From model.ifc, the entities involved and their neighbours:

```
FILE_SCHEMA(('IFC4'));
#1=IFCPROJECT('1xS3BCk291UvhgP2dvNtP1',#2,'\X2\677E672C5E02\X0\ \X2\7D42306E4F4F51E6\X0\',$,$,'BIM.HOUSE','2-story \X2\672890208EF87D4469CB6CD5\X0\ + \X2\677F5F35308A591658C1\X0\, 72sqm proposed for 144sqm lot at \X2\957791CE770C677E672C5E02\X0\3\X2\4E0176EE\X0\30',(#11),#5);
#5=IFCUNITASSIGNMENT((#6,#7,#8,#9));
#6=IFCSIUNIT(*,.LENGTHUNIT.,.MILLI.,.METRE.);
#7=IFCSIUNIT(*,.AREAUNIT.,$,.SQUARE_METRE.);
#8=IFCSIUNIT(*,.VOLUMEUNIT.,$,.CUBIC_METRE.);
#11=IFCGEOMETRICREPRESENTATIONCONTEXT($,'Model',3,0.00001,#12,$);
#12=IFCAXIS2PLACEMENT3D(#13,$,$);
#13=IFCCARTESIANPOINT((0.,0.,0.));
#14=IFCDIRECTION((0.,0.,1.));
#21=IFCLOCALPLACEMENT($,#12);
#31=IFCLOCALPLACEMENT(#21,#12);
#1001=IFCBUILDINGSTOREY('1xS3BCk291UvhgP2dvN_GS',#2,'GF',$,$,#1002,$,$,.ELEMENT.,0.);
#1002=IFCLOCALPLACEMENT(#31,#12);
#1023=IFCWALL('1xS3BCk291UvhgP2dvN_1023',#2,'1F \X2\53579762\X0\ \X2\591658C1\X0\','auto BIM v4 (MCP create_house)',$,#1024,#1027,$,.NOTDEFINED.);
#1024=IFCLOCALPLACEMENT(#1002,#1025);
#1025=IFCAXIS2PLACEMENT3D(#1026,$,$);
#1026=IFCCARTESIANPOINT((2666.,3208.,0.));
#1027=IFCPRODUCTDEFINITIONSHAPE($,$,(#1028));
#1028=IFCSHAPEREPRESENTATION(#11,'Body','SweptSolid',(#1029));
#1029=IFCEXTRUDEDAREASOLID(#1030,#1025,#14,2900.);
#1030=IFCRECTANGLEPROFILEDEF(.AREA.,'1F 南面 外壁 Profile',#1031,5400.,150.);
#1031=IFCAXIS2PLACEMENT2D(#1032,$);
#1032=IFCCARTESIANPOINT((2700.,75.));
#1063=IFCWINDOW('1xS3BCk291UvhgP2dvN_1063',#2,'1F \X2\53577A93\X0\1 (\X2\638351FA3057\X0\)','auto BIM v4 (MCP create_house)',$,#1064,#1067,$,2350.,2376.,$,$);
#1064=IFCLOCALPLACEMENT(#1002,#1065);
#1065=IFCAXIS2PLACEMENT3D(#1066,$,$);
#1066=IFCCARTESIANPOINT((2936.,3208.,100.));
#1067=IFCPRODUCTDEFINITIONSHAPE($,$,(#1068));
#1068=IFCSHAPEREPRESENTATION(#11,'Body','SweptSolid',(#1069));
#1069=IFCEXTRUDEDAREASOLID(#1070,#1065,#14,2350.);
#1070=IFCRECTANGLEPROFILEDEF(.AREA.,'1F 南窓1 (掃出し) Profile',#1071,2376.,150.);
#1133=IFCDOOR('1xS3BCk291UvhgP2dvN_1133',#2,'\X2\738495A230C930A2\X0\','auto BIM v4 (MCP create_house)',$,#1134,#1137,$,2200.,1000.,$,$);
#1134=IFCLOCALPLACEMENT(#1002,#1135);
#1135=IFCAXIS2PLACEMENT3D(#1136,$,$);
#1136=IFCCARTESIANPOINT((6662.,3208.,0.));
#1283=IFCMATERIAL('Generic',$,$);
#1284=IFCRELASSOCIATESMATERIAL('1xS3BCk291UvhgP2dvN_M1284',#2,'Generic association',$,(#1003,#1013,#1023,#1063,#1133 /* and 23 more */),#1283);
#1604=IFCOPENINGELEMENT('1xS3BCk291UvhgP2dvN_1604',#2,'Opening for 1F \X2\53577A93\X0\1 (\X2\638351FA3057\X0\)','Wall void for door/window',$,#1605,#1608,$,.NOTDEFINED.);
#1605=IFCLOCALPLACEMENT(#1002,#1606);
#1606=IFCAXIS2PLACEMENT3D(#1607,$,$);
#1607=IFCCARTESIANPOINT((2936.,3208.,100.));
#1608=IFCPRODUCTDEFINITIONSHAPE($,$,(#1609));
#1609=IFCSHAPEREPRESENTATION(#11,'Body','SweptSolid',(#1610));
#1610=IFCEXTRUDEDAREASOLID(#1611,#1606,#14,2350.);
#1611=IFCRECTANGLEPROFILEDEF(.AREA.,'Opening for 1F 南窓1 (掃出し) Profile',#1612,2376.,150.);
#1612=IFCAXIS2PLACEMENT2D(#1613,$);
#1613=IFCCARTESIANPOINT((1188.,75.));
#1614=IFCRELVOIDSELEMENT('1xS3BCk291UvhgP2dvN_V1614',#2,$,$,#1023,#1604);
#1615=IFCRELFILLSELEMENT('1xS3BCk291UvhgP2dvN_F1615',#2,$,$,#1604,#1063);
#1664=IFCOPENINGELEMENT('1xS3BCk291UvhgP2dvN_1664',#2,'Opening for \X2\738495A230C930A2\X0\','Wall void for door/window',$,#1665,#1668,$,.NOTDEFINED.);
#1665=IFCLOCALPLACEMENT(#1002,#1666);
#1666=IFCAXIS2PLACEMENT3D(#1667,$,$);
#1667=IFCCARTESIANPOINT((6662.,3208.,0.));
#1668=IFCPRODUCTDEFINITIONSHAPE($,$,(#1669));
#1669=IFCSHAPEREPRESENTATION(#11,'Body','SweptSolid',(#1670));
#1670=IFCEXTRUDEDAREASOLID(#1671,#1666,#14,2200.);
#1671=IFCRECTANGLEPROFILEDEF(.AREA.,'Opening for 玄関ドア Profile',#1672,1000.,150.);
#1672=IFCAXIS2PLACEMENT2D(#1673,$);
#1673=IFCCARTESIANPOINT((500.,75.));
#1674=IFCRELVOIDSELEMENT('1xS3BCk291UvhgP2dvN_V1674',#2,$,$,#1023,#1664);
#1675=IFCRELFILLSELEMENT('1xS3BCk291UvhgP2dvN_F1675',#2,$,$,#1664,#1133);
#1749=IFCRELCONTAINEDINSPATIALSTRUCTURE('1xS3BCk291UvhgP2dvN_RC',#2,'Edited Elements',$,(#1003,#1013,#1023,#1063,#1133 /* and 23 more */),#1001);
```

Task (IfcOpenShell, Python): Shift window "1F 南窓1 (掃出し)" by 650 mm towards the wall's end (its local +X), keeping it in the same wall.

```python
import ifcopenshell
import ifcopenshell.api.geometry
import ifcopenshell.util.placement

model = ifcopenshell.open("model.ifc")

window = model.by_id(1063)
opening = window.FillsVoids[0].RelatingOpeningElement
wall = opening.VoidsElements[0].RelatingBuildingElement

wall_matrix = ifcopenshell.util.placement.get_local_placement(wall.ObjectPlacement)
shift = wall_matrix[:3, 0] * 650.0
before = ifcopenshell.util.placement.get_local_placement(window.ObjectPlacement)[:3, 3].copy()

# The window is not placed relative to its opening, so move both.
for product in (opening, window):
    matrix = ifcopenshell.util.placement.get_local_placement(product.ObjectPlacement)
    matrix[:3, 3] += shift
    ifcopenshell.api.geometry.edit_object_placement(model, product=product, matrix=matrix, is_si=False)

after = ifcopenshell.util.placement.get_local_placement(window.ObjectPlacement)[:3, 3]
print("window moved by", (after - before).round(3) + 0.0)

model.write("model-out.ifc")
```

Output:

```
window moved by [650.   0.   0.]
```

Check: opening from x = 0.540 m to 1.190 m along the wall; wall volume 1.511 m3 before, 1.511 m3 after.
